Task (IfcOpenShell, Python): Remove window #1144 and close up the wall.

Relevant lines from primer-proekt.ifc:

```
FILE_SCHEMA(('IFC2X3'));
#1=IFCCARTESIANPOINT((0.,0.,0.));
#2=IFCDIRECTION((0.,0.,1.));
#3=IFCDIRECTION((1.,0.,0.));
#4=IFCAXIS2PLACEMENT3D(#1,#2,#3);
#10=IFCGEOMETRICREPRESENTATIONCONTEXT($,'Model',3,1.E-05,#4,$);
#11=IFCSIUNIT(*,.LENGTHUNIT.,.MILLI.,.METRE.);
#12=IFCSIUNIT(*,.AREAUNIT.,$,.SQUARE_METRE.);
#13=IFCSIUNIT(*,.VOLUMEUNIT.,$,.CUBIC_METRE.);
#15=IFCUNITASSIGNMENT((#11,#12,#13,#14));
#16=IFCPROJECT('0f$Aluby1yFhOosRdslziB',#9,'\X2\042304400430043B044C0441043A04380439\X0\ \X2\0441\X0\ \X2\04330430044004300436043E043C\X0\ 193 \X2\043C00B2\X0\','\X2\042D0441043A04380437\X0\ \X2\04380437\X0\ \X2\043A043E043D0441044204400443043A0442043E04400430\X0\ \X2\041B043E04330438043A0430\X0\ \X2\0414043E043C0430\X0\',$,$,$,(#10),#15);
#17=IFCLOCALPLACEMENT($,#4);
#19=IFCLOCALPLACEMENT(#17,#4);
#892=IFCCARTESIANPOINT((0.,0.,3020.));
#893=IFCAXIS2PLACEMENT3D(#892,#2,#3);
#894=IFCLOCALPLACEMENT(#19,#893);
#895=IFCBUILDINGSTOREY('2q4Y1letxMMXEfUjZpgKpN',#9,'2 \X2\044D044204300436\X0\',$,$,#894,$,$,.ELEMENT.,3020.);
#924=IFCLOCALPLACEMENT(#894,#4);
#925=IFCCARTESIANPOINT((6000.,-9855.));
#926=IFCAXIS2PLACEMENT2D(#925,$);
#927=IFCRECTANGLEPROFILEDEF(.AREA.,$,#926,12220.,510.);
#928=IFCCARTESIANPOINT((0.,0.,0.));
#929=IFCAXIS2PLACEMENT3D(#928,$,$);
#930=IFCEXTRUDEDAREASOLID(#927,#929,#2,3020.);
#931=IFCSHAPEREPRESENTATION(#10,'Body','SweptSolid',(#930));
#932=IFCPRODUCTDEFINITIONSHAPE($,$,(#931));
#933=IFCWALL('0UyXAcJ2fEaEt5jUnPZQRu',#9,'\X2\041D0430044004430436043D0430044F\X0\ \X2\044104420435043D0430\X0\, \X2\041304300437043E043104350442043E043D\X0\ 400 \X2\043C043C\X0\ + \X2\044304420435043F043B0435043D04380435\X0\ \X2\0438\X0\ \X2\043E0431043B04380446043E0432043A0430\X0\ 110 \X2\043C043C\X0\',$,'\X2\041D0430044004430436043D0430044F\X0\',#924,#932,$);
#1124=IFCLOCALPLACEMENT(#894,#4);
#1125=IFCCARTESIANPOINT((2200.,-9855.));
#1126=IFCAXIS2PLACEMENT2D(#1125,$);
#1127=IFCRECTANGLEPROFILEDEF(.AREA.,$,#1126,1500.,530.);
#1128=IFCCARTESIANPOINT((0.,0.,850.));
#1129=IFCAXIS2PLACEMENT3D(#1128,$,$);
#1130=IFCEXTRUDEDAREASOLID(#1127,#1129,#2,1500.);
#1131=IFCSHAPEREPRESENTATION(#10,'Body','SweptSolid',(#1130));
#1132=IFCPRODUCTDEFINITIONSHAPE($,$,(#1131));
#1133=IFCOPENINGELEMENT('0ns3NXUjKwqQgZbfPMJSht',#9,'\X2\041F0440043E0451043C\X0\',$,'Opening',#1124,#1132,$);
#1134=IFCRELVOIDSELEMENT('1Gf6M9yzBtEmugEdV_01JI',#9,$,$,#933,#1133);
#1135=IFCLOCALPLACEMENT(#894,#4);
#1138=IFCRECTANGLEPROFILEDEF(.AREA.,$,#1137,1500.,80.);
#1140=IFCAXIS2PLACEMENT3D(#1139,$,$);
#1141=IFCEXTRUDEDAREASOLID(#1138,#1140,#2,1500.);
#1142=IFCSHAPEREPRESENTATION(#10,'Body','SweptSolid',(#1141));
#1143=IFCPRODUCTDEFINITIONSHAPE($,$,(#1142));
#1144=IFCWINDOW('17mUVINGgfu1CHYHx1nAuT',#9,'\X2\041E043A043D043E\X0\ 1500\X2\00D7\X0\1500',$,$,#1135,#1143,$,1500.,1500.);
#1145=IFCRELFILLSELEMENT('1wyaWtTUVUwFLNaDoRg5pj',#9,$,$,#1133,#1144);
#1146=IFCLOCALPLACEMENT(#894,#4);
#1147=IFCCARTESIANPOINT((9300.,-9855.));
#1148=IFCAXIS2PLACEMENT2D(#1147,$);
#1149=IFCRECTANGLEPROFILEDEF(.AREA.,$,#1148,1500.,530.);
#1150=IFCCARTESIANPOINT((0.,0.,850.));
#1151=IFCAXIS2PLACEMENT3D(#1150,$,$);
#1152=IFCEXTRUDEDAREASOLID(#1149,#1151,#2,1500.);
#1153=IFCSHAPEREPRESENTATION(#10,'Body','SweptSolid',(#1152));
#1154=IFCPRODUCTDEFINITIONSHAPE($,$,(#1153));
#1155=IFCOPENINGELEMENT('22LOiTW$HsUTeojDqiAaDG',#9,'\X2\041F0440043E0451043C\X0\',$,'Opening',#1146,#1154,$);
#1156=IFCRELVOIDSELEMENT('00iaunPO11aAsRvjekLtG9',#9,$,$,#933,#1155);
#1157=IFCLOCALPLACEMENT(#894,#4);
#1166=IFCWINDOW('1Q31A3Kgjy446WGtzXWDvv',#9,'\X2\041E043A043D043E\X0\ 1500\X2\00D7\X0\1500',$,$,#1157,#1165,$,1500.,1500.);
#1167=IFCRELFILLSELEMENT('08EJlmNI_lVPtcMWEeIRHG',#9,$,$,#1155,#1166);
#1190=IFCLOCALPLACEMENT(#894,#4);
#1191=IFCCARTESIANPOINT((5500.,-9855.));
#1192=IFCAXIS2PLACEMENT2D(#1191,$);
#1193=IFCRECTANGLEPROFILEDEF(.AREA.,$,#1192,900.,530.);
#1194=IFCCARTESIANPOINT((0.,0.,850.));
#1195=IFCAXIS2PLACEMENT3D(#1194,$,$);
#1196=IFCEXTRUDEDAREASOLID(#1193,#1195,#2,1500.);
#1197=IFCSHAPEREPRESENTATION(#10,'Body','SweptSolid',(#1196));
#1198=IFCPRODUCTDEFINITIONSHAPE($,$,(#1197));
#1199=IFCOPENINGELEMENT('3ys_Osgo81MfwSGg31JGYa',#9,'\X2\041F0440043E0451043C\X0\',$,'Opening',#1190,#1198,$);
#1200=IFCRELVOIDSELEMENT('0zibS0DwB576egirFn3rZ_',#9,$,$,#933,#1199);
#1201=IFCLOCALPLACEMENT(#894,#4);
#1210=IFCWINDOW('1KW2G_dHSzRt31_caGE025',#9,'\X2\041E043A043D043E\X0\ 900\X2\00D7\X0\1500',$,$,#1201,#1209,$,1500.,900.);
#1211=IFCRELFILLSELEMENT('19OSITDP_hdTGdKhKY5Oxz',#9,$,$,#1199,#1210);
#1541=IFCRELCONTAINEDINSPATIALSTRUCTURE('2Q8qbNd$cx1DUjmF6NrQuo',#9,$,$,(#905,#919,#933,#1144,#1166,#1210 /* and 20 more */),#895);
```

```python
import ifcopenshell
import ifcopenshell.api.feature
import ifcopenshell.api.root
import ifcopenshell.geom
import ifcopenshell.util.shape

model = ifcopenshell.open("primer-proekt.ifc")
settings = ifcopenshell.geom.settings()


def volume(element):
    """Net volume in cubic metres, openings subtracted."""
    shape = ifcopenshell.geom.create_shape(settings, element)
    return ifcopenshell.util.shape.get_volume(shape.geometry)


window = model.by_guid("17mUVINGgfu1CHYHx1nAuT")
opening = window.FillsVoids[0].RelatingOpeningElement
wall = opening.VoidsElements[0].RelatingBuildingElement
before = volume(wall)

ifcopenshell.api.root.remove_product(model, product=window)
ifcopenshell.api.feature.remove_feature(model, feature=opening)

after = volume(wall)

print(f"wall volume {before:.3f} -> {after:.3f} m3")

model.write("primer-proekt_edited.ifc")
```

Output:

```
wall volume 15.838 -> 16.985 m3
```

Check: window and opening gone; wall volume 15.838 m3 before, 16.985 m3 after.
